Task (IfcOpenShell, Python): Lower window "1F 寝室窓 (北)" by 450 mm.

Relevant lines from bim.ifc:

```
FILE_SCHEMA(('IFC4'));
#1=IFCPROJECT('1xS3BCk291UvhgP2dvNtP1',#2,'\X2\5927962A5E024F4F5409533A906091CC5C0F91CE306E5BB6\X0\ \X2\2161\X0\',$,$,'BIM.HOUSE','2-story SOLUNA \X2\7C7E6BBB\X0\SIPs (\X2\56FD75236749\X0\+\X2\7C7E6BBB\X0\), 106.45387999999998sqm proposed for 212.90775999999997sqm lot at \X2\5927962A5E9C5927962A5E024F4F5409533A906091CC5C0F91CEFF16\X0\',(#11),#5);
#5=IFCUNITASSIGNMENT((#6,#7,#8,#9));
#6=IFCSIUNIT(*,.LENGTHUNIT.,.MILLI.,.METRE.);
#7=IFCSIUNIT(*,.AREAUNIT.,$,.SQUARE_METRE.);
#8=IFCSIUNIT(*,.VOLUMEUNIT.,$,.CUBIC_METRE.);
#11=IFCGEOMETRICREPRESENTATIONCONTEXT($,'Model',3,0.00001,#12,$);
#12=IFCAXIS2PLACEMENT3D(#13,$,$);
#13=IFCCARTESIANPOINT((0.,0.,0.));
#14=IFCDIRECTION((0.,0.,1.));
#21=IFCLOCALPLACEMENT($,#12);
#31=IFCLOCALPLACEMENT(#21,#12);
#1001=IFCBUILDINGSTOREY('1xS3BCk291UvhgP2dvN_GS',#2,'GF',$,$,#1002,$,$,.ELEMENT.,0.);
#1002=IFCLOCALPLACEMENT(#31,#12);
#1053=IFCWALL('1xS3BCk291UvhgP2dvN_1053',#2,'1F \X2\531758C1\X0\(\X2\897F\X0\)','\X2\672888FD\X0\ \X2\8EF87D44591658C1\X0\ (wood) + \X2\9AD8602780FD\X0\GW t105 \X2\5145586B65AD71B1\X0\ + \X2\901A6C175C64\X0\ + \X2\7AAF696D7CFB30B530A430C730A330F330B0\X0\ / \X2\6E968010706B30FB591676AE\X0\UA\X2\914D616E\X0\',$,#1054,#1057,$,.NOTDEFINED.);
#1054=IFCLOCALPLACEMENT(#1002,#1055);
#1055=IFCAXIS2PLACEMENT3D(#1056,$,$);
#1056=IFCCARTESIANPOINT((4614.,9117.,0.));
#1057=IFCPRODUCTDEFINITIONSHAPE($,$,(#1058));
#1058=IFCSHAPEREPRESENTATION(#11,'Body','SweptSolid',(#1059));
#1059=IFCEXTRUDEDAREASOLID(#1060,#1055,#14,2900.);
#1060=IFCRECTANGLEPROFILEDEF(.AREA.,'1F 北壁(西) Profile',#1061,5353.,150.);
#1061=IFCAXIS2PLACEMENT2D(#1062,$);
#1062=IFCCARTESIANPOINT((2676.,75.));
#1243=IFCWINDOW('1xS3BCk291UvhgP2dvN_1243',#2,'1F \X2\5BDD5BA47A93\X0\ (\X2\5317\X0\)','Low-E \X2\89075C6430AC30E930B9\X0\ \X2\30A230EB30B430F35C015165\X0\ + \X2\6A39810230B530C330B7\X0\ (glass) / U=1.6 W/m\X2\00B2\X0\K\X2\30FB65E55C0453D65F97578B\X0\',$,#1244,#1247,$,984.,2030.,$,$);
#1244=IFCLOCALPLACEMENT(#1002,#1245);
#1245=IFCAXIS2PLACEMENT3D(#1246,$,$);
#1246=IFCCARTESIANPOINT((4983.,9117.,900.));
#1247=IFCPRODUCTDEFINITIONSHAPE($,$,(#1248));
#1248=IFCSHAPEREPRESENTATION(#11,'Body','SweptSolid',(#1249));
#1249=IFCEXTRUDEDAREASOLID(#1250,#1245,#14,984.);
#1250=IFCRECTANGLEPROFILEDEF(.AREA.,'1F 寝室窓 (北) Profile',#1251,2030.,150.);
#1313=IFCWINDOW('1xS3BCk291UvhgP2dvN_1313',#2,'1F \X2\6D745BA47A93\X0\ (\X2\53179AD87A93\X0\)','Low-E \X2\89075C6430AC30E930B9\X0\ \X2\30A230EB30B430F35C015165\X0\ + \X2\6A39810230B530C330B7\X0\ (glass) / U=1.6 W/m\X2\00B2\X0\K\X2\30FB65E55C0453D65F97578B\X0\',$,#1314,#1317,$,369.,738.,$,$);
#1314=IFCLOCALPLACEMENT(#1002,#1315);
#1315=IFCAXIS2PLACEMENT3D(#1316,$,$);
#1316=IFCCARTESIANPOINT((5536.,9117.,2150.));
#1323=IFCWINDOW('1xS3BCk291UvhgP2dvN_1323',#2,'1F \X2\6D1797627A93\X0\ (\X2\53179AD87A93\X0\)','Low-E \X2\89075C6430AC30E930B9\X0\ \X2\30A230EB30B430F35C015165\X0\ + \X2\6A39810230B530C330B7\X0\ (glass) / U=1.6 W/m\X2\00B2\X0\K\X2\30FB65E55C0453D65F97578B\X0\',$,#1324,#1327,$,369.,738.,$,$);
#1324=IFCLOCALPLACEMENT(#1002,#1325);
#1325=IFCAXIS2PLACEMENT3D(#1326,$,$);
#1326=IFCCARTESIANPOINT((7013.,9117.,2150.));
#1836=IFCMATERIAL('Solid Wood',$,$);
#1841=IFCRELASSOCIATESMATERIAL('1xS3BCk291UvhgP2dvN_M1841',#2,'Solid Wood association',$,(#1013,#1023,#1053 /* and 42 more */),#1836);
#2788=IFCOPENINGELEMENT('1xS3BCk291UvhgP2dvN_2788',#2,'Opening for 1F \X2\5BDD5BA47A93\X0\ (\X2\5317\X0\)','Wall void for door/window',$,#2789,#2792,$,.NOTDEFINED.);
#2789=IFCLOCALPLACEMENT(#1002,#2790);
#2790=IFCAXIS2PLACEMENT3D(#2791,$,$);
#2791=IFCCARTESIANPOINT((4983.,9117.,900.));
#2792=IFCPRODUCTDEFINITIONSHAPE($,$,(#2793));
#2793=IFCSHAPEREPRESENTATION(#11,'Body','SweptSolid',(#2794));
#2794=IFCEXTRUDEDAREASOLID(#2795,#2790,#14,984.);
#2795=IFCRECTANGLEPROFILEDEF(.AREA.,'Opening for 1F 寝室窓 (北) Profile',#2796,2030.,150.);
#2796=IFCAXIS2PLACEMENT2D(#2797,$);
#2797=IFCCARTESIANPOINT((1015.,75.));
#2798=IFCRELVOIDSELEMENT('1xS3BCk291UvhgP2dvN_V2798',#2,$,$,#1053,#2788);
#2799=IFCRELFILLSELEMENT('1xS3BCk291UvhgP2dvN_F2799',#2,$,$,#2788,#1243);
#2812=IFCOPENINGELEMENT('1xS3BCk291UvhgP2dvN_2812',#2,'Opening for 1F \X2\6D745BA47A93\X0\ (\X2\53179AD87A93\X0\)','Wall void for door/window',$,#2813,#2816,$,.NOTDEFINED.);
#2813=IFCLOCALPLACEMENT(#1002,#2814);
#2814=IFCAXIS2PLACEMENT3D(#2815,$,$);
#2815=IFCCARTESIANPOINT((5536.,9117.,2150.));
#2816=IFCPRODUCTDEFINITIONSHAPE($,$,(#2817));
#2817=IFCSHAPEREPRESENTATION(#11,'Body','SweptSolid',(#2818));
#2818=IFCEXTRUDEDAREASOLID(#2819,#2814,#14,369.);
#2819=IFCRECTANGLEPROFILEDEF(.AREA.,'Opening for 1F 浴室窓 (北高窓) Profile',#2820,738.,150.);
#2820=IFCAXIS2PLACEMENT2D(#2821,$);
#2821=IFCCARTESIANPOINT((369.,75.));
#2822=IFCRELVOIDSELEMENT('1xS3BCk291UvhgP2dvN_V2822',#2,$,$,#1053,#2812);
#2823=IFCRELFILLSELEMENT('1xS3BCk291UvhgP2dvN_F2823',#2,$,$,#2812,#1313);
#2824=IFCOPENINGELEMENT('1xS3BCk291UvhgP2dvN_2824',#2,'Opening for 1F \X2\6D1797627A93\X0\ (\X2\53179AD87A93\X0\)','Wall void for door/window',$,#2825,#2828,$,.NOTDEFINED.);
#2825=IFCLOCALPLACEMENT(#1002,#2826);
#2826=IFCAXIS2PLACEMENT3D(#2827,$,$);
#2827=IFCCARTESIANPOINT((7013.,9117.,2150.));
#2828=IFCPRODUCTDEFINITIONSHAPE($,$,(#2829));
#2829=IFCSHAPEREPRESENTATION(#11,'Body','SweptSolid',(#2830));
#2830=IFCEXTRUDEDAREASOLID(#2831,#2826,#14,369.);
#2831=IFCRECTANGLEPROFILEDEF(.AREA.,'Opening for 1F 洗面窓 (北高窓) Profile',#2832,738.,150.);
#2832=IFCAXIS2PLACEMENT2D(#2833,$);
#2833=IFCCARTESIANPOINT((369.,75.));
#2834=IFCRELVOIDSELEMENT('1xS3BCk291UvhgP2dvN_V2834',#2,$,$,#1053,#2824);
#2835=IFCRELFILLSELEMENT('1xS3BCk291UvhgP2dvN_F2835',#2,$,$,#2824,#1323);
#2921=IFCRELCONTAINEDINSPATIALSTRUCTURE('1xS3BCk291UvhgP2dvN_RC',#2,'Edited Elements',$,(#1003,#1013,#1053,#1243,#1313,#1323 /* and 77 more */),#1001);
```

```python
import numpy as np
import ifcopenshell
import ifcopenshell.api.geometry
import ifcopenshell.util.placement
import ifcopenshell.util.unit

model = ifcopenshell.open("bim.ifc")
unit_scale = ifcopenshell.util.unit.calculate_unit_scale(model)

window = model.by_guid("1xS3BCk291UvhgP2dvN_1243")
opening = window.FillsVoids[0].RelatingOpeningElement
dz = -450.0

shift = np.array([0.0, 0.0, dz])
# The window is not placed relative to its opening, so move both.
for product in (opening, window):
    matrix = ifcopenshell.util.placement.get_local_placement(product.ObjectPlacement)
    matrix[:3, 3] += shift
    ifcopenshell.api.geometry.edit_object_placement(model, product=product, matrix=matrix, is_si=False)

print(f"moved by {dz * unit_scale:+.3f} m")

model.write("bim-out.ifc")
```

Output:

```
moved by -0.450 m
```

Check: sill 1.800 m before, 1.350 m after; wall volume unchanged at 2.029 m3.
